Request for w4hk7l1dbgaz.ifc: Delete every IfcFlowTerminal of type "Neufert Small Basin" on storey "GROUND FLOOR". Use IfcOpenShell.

First a look at what the model holds.

```python
import ifcopenshell
import ifcopenshell.util.element

model = ifcopenshell.open("w4hk7l1dbgaz.ifc")
print(model.schema)
storey = next(s for s in model.by_type("IfcBuildingStorey") if s.Name == "GROUND FLOOR")
terminals = [e for e in ifcopenshell.util.element.get_decomposition(storey) if e.is_a("IfcFlowTerminal")]
seen = {}
for e in terminals:
    element_type = ifcopenshell.util.element.get_type(e)
    name = element_type.Name if element_type not in (None, e) else None
    seen[name] = seen.get(name, 0) + 1
for name, count in sorted(seen.items(), key=str):
    print(count, "x", name)
```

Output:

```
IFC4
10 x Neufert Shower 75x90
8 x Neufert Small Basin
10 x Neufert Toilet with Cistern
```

```python
import ifcopenshell
import ifcopenshell.api.root
import ifcopenshell.util.element

model = ifcopenshell.open("w4hk7l1dbgaz.ifc")

storey = next(s for s in model.by_type("IfcBuildingStorey") if s.Name == "GROUND FLOOR")
terminals = [e for e in ifcopenshell.util.element.get_decomposition(storey) if e.is_a("IfcFlowTerminal")]
targets = [e for e in terminals if (t := ifcopenshell.util.element.get_type(e)) not in (None, e) and t.Name == "Neufert Small Basin"]

for e in targets:
    ifcopenshell.api.root.remove_product(model, product=e)
print(len(targets), "removed")

model.write("w4hk7l1dbgaz-out.ifc")
```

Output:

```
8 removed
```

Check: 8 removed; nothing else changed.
